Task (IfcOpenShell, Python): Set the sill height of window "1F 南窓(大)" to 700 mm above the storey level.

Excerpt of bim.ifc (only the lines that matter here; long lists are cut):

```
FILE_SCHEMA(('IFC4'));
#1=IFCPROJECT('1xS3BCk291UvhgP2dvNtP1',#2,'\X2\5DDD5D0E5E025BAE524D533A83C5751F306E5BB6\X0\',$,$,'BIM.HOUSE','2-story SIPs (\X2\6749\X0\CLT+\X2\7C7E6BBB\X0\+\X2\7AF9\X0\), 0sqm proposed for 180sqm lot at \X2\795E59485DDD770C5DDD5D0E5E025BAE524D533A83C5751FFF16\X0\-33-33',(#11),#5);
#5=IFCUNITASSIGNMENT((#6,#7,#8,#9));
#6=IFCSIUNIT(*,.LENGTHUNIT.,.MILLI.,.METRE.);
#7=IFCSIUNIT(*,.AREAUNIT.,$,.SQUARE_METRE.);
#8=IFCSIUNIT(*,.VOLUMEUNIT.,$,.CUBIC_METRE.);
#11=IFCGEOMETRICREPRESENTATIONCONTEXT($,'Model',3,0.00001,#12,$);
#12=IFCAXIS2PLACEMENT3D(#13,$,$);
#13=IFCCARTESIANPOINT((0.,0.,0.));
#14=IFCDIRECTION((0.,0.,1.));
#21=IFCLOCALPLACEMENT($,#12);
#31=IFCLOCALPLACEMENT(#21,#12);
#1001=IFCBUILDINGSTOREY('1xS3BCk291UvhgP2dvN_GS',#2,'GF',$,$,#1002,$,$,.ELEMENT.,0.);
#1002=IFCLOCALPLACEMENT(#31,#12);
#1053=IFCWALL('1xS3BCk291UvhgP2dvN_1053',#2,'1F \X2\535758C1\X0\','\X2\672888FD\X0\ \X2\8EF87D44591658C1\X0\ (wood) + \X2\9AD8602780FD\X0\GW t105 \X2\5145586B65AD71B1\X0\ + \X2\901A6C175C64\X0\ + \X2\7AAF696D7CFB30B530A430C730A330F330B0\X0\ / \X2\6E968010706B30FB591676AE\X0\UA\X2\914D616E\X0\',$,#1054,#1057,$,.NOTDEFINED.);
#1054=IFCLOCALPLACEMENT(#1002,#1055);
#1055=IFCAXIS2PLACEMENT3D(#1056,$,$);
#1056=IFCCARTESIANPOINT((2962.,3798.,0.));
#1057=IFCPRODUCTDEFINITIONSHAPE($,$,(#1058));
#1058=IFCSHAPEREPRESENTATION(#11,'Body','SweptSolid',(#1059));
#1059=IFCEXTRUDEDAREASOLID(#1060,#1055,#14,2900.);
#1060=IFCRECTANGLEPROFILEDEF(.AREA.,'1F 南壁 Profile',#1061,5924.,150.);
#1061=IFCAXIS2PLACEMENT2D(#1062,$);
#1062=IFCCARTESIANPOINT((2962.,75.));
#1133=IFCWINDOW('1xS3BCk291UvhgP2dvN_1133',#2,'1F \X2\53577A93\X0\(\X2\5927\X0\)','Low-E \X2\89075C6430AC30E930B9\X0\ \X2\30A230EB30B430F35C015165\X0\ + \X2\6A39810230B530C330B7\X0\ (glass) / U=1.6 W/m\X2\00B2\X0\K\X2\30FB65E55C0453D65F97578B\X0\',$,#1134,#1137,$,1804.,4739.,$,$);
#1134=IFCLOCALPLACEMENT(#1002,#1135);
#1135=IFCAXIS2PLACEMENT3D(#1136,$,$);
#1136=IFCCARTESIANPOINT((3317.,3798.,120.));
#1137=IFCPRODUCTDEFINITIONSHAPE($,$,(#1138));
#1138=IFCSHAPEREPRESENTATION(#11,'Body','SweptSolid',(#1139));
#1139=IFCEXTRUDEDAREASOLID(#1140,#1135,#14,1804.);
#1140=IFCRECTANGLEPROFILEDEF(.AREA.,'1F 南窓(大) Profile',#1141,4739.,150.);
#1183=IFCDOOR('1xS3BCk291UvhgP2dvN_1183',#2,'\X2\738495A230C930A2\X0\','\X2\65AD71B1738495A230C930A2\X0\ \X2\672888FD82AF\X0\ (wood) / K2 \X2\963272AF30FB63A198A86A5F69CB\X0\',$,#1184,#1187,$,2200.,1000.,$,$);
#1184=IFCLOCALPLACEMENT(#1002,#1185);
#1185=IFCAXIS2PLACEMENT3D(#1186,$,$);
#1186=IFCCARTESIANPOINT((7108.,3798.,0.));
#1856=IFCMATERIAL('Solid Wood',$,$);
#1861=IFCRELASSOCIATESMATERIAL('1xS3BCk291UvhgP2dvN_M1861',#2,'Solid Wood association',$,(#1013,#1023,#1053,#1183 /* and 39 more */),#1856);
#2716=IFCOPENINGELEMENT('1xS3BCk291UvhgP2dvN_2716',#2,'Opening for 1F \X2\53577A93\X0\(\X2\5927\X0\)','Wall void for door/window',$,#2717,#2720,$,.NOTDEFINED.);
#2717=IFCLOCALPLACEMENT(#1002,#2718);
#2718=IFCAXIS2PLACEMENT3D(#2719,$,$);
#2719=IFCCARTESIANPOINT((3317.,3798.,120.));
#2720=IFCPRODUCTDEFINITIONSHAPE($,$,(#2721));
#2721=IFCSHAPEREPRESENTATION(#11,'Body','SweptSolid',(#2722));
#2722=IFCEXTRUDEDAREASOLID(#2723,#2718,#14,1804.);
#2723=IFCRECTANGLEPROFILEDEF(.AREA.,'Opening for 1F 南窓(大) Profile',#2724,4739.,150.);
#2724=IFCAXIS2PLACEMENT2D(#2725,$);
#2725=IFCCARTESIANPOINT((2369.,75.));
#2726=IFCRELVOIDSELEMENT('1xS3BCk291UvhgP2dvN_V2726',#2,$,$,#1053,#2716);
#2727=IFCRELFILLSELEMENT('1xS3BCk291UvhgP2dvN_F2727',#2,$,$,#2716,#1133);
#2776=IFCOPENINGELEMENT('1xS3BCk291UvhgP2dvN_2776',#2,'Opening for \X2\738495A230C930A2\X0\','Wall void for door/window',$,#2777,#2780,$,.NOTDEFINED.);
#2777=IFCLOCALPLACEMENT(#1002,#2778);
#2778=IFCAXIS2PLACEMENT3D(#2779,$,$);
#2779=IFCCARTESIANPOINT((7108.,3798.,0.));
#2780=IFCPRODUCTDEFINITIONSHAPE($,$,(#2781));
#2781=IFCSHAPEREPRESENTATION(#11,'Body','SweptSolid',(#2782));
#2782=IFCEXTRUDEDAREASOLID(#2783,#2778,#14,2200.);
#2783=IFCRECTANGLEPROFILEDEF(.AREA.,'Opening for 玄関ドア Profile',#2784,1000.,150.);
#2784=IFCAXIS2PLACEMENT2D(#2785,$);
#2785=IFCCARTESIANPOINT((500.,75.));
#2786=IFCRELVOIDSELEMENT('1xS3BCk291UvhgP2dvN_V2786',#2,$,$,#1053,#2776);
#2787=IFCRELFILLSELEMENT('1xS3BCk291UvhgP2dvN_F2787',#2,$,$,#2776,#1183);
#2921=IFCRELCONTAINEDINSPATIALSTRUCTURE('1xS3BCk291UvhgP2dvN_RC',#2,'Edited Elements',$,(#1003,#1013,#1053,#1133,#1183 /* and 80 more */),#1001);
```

```python
import numpy as np
import ifcopenshell
import ifcopenshell.api.geometry
import ifcopenshell.geom
import ifcopenshell.util.element
import ifcopenshell.util.placement
import ifcopenshell.util.shape
import ifcopenshell.util.unit

model = ifcopenshell.open("bim.ifc")
unit_scale = ifcopenshell.util.unit.calculate_unit_scale(model)

window = model.by_guid("1xS3BCk291UvhgP2dvN_1133")
opening = window.FillsVoids[0].RelatingOpeningElement
storey = ifcopenshell.util.element.get_container(window, ifc_class="IfcBuildingStorey")
level = ifcopenshell.util.placement.get_local_placement(storey.ObjectPlacement)[2, 3]

# The opening's origin need not be at the sill, so measure its lowest point.
shape = ifcopenshell.geom.create_shape(ifcopenshell.geom.settings(), opening)
bottom = ifcopenshell.util.shape.get_shape_bottom_elevation(shape, shape.geometry) / unit_scale
dz = level + 0.7 / unit_scale - bottom

shift = np.array([0.0, 0.0, dz])
# The window is not placed relative to its opening, so move both.
for product in (opening, window):
    matrix = ifcopenshell.util.placement.get_local_placement(product.ObjectPlacement)
    matrix[:3, 3] += shift
    ifcopenshell.api.geometry.edit_object_placement(model, product=product, matrix=matrix, is_si=False)

print(f"moved by {dz * unit_scale:+.3f} m")

model.write("bim-out.ifc")
```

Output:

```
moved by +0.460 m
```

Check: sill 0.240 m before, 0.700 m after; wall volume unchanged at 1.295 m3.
